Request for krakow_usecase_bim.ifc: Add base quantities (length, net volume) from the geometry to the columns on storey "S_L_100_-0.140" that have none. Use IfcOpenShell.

First a look at what the model holds.

```python
import ifcopenshell
import ifcopenshell.util.element
import ifcopenshell.util.unit

model = ifcopenshell.open("krakow_usecase_bim.ifc")
print(model.schema)
for unit_type in ("LENGTHUNIT", "AREAUNIT", "VOLUMEUNIT"):
    print(unit_type, ifcopenshell.util.unit.calculate_unit_scale(model, unit_type))
storey = next(s for s in model.by_type("IfcBuildingStorey") if s.Name == "S_L_100_-0.140")
columns = [e for e in ifcopenshell.util.element.get_decomposition(storey) if e.is_a("IfcColumn")]
for e in sorted(columns, key=lambda e: e.id()):
    print(e.id(), e.is_a(), e.Name, list(ifcopenshell.util.element.get_psets(e, qtos_only=True)), sep=" | ")
```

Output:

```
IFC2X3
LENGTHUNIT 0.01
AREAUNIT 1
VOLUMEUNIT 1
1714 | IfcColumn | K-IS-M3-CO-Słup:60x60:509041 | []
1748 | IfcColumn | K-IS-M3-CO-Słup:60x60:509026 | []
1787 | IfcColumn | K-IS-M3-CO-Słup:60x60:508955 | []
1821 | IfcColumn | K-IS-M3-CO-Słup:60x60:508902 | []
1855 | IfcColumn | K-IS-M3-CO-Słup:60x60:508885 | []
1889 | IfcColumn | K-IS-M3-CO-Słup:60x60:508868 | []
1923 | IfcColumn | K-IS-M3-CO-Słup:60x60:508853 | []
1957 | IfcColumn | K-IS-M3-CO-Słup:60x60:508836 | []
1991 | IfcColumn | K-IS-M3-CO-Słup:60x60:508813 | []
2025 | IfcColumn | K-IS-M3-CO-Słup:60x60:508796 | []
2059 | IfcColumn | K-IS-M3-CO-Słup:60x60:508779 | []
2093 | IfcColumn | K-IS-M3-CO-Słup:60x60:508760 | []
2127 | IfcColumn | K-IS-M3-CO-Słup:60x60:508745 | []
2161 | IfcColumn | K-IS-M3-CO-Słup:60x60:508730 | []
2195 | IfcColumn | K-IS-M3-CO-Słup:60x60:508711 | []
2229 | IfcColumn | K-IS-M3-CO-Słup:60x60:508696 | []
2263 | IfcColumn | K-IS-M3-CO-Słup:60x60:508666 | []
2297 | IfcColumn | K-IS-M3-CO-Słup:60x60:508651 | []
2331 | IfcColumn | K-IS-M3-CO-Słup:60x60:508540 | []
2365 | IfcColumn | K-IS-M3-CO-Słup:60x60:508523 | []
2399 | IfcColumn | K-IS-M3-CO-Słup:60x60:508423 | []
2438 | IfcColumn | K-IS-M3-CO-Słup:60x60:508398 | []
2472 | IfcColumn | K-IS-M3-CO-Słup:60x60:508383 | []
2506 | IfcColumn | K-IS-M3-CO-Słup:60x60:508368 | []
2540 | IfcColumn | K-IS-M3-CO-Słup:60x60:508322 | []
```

```python
import ifcopenshell
import ifcopenshell.api.pset
import ifcopenshell.geom
import ifcopenshell.util.element
import ifcopenshell.util.shape
import ifcopenshell.util.unit

model = ifcopenshell.open("krakow_usecase_bim.ifc")
unit_scale = ifcopenshell.util.unit.calculate_unit_scale(model)
volume_scale = ifcopenshell.util.unit.calculate_unit_scale(model, "VOLUMEUNIT")
settings = ifcopenshell.geom.settings()

storey = next(s for s in model.by_type("IfcBuildingStorey") if s.Name == "S_L_100_-0.140")
columns = [e for e in ifcopenshell.util.element.get_decomposition(storey) if e.is_a("IfcColumn")]

for e in sorted(columns, key=lambda e: e.id()):
    if ifcopenshell.util.element.get_psets(e, qtos_only=True, should_inherit=False):
        continue
    # Geometry comes back in metres, in the element's own axes.
    shape = ifcopenshell.geom.create_shape(settings, e)
    values = {
        "Length": ifcopenshell.util.shape.get_z(shape.geometry) / unit_scale,
        "NetVolume": ifcopenshell.util.shape.get_volume(shape.geometry) / volume_scale,
    }
    qto = ifcopenshell.api.pset.add_qto(model, product=e, name="BaseQuantities")
    ifcopenshell.api.pset.edit_qto(model, qto=qto, properties=values)
    print(e.id(), {k: round(v, 3) for k, v in values.items()})

model.write("krakow_usecase_bim-out.ifc")
```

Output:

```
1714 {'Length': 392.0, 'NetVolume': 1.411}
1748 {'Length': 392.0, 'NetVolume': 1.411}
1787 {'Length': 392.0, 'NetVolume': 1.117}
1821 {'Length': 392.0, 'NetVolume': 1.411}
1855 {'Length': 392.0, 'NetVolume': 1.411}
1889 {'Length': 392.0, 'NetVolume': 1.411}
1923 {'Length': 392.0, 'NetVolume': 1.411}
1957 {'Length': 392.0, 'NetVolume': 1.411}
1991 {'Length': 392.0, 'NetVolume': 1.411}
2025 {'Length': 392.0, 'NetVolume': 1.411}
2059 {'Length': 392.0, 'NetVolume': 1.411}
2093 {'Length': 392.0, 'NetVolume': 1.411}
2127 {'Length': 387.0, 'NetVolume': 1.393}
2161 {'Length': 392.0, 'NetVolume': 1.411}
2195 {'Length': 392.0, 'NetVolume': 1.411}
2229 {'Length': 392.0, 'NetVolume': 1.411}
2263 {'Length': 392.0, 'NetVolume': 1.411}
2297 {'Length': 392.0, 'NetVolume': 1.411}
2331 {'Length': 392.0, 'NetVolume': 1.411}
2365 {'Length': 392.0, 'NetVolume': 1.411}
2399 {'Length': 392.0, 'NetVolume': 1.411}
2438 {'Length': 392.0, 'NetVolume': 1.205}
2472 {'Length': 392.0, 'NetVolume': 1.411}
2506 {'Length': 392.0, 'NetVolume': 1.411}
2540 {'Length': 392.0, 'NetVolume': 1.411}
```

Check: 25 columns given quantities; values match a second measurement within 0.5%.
